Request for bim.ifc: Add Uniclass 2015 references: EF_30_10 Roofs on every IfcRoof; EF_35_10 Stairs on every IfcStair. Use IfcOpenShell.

First a look at what the model holds.

```python
import ifcopenshell

model = ifcopenshell.open("bim.ifc")
print(model.schema)
print("classifications:", [c.Name for c in model.by_type("IfcClassification")])
for ifc_class in ("IfcDoor", "IfcRoof", "IfcStair", "IfcWall", "IfcWindow"):
    print(ifc_class, len(model.by_type(ifc_class)))
```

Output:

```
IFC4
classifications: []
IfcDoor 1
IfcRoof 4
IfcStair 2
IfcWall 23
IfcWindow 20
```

```python
import ifcopenshell
import ifcopenshell.api.classification

model = ifcopenshell.open("bim.ifc")

system = ifcopenshell.api.classification.add_classification(model, classification="Uniclass 2015")

codes = {
    "IfcRoof": ("EF_30_10", "Roofs"),
    "IfcStair": ("EF_35_10", "Stairs"),
}
for ifc_class, (code, name) in codes.items():
    products = model.by_type(ifc_class)
    ifcopenshell.api.classification.add_reference(
        model, products=products, classification=system, identification=code, name=name
    )
    print(code, len(products))

model.write("bim_v2.ifc")
```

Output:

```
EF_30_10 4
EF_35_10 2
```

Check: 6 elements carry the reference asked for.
